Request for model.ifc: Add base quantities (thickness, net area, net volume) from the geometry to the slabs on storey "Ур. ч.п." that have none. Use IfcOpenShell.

First a look at what the model holds.

```python
import ifcopenshell
import ifcopenshell.util.element
import ifcopenshell.util.unit

model = ifcopenshell.open("model.ifc")
print(model.schema)
for unit_type in ("LENGTHUNIT", "AREAUNIT", "VOLUMEUNIT"):
    print(unit_type, ifcopenshell.util.unit.calculate_unit_scale(model, unit_type))
storey = next(s for s in model.by_type("IfcBuildingStorey") if s.Name == "Ур. ч.п.")
slabs = [e for e in ifcopenshell.util.element.get_decomposition(storey) if e.is_a("IfcSlab")]
for e in sorted(slabs, key=lambda e: e.id()):
    print(e.id(), e.is_a(), e.Name, list(ifcopenshell.util.element.get_psets(e, qtos_only=True)), sep=" | ")
```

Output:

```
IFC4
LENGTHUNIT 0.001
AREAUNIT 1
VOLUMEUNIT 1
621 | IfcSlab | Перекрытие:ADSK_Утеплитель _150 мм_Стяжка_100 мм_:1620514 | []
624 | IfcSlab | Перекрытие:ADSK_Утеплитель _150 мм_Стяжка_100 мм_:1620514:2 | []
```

```python
import ifcopenshell
import ifcopenshell.api.pset
import ifcopenshell.geom
import ifcopenshell.util.element
import ifcopenshell.util.shape
import ifcopenshell.util.unit

model = ifcopenshell.open("model.ifc")
unit_scale = ifcopenshell.util.unit.calculate_unit_scale(model)
area_scale = ifcopenshell.util.unit.calculate_unit_scale(model, "AREAUNIT")
volume_scale = ifcopenshell.util.unit.calculate_unit_scale(model, "VOLUMEUNIT")
settings = ifcopenshell.geom.settings()

storey = next(s for s in model.by_type("IfcBuildingStorey") if s.Name == "Ур. ч.п.")
slabs = [e for e in ifcopenshell.util.element.get_decomposition(storey) if e.is_a("IfcSlab")]

for e in sorted(slabs, key=lambda e: e.id()):
    if ifcopenshell.util.element.get_psets(e, qtos_only=True, should_inherit=False):
        continue
    # Geometry comes back in metres, in the element's own axes.
    shape = ifcopenshell.geom.create_shape(settings, e)
    values = {
        "Width": ifcopenshell.util.shape.get_z(shape.geometry) / unit_scale,
        "NetArea": ifcopenshell.util.shape.get_footprint_area(shape.geometry) / area_scale,
        "NetVolume": ifcopenshell.util.shape.get_volume(shape.geometry) / volume_scale,
    }
    qto = ifcopenshell.api.pset.add_qto(model, product=e, name="Qto_SlabBaseQuantities")
    ifcopenshell.api.pset.edit_qto(model, qto=qto, properties=values)
    print(e.id(), {k: round(v, 3) for k, v in values.items()})

model.write("model_edited.ifc")
```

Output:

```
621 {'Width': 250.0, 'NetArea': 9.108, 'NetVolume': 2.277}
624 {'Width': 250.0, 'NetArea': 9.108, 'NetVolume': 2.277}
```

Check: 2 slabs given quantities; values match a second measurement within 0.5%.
